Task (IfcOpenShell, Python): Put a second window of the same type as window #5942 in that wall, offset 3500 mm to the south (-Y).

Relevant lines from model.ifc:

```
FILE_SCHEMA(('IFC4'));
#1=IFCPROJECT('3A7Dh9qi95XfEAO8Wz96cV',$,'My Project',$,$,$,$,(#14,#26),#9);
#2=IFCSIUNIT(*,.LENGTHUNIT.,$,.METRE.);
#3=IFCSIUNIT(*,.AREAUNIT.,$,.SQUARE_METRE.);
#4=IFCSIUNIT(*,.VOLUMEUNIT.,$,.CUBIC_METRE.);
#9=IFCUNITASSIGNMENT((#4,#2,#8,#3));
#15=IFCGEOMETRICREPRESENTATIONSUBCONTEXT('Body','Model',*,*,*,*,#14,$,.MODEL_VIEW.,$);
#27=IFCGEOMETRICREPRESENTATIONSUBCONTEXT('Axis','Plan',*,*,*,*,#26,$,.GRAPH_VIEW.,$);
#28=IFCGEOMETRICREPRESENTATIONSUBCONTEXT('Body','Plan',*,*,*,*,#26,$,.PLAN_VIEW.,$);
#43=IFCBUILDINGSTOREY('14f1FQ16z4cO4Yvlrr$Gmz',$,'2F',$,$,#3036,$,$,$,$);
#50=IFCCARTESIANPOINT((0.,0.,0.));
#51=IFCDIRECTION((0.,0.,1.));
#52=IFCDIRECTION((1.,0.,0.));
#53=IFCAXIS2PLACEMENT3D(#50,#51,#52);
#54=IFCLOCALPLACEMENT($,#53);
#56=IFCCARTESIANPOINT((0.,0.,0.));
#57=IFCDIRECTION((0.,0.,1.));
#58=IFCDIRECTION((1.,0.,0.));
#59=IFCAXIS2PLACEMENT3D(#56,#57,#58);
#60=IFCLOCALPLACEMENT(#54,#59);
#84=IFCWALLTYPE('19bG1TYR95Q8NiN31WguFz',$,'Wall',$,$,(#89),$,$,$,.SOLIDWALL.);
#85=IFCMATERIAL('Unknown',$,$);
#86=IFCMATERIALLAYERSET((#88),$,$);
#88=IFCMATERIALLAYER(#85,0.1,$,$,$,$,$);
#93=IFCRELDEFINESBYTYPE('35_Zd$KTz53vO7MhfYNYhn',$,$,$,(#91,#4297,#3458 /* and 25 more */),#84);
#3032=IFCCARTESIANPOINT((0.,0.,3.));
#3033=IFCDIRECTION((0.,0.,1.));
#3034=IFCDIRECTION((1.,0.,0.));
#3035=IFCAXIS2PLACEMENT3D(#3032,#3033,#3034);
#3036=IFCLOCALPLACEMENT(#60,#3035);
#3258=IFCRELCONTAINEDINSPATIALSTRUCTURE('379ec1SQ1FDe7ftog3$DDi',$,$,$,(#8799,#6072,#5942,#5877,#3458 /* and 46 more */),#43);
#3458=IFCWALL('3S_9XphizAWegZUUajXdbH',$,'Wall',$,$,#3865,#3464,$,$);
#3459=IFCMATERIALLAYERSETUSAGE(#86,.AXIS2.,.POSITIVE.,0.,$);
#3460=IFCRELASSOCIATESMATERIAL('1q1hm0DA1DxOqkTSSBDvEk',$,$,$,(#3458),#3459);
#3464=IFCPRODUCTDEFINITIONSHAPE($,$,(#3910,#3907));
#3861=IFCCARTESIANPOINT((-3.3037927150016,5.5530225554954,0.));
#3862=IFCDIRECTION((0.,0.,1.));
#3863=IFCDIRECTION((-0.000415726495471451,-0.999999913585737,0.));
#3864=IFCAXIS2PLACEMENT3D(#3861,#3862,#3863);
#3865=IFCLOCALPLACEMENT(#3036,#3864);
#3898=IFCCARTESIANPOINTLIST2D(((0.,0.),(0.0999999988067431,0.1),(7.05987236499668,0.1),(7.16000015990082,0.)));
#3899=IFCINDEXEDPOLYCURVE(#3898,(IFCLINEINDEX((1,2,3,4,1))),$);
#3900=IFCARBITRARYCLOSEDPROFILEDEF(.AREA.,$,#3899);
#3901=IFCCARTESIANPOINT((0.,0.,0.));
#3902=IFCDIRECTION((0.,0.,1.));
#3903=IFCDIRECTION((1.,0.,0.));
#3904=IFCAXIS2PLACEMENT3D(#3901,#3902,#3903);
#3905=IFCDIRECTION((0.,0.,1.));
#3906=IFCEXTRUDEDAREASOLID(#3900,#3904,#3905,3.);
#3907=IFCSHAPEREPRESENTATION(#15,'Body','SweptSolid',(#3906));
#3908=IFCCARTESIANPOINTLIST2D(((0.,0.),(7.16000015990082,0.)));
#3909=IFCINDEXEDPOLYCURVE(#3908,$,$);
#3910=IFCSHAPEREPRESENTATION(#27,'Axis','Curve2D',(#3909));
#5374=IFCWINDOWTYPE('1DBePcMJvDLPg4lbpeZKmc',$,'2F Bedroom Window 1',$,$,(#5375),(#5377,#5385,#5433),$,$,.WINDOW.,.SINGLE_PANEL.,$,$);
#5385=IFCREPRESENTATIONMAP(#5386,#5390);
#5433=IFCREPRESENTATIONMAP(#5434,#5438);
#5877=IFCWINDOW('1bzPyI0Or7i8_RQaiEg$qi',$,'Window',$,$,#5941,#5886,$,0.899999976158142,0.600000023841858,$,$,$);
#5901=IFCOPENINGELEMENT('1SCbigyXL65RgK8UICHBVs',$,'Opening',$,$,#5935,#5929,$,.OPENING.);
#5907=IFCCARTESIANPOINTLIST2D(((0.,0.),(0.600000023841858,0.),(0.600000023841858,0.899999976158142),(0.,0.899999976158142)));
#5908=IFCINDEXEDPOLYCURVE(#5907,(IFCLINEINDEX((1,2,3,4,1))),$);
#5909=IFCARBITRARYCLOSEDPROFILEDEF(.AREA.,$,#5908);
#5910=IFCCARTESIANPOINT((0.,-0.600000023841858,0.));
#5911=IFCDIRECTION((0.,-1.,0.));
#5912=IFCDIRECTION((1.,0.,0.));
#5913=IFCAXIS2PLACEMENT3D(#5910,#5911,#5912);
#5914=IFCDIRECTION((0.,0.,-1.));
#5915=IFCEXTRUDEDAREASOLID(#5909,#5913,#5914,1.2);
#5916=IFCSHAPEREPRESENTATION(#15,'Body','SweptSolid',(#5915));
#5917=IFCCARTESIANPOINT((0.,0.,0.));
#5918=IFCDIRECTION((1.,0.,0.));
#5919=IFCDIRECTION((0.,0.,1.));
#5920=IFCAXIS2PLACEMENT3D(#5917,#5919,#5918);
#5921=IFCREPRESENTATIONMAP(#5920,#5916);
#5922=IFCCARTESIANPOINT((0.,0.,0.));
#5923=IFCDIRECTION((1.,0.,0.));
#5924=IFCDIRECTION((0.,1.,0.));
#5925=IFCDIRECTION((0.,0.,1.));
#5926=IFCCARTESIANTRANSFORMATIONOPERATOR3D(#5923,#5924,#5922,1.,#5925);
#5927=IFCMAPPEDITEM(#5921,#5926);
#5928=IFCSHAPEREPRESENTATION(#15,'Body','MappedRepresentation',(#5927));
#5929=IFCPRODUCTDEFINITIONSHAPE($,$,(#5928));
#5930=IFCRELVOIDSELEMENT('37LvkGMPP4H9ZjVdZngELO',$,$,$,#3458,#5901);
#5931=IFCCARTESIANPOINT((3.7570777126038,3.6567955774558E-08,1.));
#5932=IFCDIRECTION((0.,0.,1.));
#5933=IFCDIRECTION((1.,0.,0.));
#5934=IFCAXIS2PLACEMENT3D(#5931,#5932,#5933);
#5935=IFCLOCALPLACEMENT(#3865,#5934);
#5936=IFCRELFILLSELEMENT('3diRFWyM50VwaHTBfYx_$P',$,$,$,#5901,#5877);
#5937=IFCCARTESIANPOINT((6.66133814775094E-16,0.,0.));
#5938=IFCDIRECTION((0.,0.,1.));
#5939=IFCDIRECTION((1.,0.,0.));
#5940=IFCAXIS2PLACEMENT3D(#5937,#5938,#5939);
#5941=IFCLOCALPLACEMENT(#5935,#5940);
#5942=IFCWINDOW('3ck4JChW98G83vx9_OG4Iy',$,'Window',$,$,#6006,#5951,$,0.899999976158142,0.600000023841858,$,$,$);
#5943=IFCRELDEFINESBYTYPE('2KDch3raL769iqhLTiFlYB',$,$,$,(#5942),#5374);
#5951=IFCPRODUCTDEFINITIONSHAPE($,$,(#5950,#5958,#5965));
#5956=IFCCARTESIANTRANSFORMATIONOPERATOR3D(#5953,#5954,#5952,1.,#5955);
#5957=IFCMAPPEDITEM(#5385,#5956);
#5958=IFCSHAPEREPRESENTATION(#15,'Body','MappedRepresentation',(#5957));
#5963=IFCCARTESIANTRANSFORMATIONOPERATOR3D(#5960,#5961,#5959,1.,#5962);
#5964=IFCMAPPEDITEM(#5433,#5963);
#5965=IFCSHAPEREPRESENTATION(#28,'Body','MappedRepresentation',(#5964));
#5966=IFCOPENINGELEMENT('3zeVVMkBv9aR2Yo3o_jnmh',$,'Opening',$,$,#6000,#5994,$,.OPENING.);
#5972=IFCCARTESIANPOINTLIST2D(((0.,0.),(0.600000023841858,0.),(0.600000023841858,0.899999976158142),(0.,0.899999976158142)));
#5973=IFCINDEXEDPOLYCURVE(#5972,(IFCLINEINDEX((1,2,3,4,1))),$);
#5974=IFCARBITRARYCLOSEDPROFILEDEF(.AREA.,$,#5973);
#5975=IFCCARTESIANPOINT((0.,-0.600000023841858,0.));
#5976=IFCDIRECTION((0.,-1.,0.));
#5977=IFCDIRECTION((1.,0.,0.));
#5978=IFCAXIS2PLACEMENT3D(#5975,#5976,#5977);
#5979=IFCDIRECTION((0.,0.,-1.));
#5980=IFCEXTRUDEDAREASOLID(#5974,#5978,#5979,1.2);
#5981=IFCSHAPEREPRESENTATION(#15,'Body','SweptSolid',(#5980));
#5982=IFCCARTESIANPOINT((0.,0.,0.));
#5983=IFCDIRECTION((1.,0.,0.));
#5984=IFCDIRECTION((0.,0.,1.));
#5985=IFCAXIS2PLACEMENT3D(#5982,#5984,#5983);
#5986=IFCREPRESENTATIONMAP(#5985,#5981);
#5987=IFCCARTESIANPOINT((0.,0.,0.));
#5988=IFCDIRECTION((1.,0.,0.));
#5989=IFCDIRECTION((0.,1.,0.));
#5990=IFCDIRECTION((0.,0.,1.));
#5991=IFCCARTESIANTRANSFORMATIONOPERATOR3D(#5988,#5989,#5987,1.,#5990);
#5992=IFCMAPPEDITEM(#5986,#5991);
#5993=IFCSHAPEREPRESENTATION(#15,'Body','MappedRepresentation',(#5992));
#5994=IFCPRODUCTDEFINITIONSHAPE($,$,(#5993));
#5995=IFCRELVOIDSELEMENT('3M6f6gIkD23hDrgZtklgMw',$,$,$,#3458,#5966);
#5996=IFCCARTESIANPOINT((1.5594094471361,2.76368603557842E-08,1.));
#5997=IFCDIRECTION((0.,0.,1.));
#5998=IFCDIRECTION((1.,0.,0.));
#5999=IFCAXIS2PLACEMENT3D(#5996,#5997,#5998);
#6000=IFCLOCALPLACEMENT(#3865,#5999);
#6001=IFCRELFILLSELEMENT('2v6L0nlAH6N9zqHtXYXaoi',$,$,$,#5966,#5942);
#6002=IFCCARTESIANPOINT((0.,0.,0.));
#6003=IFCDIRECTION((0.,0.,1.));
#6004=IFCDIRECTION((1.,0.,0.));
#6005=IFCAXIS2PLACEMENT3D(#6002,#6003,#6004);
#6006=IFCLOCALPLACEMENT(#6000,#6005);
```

```python
import ifcopenshell
import ifcopenshell.api.feature
import ifcopenshell.api.geometry
import ifcopenshell.api.root
import ifcopenshell.geom
import ifcopenshell.util.element
import ifcopenshell.util.placement
import ifcopenshell.util.shape

model = ifcopenshell.open("model.ifc")
settings = ifcopenshell.geom.settings()


def volume(element):
    """Net volume in cubic metres, openings subtracted."""
    shape = ifcopenshell.geom.create_shape(settings, element)
    return ifcopenshell.util.shape.get_volume(shape.geometry)


window = model.by_guid("3ck4JChW98G83vx9_OG4Iy")
opening = window.FillsVoids[0].RelatingOpeningElement
wall = opening.VoidsElements[0].RelatingBuildingElement
before = volume(wall)
shift = ifcopenshell.util.placement.get_local_placement(wall.ObjectPlacement)[:3, 0] * 3.5

# copy_class copies the void relationship, type, container and properties, but no geometry.
new_opening = ifcopenshell.api.root.copy_class(model, product=opening)
new_opening.Representation = ifcopenshell.util.element.copy_deep(
    model, opening.Representation, exclude=["IfcGeometricRepresentationContext", "IfcRepresentationMap"]
)
new_window = ifcopenshell.api.root.copy_class(model, product=window)
new_window.Representation = ifcopenshell.util.element.copy_deep(
    model, window.Representation, exclude=["IfcGeometricRepresentationContext", "IfcRepresentationMap"]
)
ifcopenshell.api.feature.add_filling(model, opening=new_opening, element=new_window)

for old, new in ((opening, new_opening), (window, new_window)):
    matrix = ifcopenshell.util.placement.get_local_placement(old.ObjectPlacement)
    matrix[:3, 3] += shift
    ifcopenshell.api.geometry.edit_object_placement(model, product=new, matrix=matrix, is_si=False)

after = volume(wall)

print(f"wall volume {before:.3f} -> {after:.3f} m3")

model.write("model-out.ifc")
```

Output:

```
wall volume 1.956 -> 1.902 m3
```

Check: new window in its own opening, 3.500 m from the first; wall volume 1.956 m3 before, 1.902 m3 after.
